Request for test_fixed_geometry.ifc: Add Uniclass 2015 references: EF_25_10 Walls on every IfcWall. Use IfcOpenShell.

First a look at what the model holds.

```python
import ifcopenshell

model = ifcopenshell.open("test_fixed_geometry.ifc")
print(model.schema)
print("classifications:", [c.Name for c in model.by_type("IfcClassification")])
for ifc_class in ("IfcDoor", "IfcRoof", "IfcStair", "IfcWall", "IfcWindow"):
    print(ifc_class, len(model.by_type(ifc_class)))
```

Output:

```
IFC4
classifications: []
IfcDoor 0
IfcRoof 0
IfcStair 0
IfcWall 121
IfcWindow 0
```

```python
import ifcopenshell
import ifcopenshell.api.classification

model = ifcopenshell.open("test_fixed_geometry.ifc")

system = ifcopenshell.api.classification.add_classification(model, classification="Uniclass 2015")

codes = {
    "IfcWall": ("EF_25_10", "Walls"),
}
for ifc_class, (code, name) in codes.items():
    products = model.by_type(ifc_class)
    ifcopenshell.api.classification.add_reference(
        model, products=products, classification=system, identification=code, name=name
    )
    print(code, len(products))

model.write("test_fixed_geometry-out.ifc")
```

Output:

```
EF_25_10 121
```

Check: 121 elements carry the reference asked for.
